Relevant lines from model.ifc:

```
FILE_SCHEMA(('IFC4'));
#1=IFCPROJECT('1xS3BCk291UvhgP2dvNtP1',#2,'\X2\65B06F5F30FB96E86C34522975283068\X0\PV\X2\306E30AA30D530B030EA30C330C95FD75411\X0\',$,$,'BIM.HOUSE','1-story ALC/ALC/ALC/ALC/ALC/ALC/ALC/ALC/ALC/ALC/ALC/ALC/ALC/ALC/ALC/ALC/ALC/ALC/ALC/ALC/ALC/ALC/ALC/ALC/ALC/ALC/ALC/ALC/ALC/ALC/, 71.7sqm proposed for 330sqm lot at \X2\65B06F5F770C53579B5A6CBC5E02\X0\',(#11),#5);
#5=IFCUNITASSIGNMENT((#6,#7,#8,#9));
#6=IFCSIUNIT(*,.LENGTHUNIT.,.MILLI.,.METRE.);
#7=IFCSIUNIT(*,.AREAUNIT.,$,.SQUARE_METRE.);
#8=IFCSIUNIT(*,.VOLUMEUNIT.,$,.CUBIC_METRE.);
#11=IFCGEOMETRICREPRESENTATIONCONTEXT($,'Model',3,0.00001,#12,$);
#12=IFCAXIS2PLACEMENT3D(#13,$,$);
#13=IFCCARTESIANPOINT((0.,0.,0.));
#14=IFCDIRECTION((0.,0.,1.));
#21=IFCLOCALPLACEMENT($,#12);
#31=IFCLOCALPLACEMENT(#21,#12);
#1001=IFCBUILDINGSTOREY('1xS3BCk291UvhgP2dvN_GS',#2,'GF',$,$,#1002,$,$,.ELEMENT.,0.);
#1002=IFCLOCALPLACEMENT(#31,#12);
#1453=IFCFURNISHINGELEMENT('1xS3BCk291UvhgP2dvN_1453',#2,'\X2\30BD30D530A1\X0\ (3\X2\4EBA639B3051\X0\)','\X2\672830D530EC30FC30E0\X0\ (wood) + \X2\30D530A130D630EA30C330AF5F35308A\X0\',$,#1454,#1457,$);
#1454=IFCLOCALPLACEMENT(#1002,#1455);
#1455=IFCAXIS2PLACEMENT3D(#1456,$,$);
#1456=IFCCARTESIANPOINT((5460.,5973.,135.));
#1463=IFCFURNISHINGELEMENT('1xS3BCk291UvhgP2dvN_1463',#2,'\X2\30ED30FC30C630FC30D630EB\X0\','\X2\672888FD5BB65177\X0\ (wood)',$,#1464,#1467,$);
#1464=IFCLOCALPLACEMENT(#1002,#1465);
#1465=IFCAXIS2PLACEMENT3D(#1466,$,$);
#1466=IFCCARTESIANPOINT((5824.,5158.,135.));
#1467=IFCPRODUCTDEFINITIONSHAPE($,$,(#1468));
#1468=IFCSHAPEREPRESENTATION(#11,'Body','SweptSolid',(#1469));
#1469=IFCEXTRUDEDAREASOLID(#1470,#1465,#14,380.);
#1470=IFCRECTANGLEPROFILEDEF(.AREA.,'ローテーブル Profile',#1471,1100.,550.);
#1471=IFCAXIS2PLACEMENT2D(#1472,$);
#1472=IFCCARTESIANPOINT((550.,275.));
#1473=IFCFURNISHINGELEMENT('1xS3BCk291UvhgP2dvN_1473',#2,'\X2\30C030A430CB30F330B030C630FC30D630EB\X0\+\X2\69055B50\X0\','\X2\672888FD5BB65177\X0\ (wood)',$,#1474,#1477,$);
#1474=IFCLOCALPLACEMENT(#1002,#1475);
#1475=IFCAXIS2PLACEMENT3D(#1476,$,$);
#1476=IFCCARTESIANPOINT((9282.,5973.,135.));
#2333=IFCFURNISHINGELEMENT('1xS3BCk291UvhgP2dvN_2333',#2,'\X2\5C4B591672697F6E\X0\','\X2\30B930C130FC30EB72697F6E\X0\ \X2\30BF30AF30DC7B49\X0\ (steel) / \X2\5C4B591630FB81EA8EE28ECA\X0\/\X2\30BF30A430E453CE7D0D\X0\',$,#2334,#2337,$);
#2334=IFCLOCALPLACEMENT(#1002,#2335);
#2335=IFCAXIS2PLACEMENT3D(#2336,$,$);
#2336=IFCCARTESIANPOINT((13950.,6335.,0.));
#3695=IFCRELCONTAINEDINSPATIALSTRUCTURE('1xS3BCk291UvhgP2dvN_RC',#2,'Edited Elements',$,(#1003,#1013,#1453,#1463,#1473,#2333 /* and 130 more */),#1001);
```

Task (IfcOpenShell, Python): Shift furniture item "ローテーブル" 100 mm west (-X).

```python
import ifcopenshell
import ifcopenshell.api.geometry
import ifcopenshell.util.placement
import ifcopenshell.util.unit

model = ifcopenshell.open("model.ifc")
unit_scale = ifcopenshell.util.unit.calculate_unit_scale(model)

item = model.by_id(1463)
matrix = ifcopenshell.util.placement.get_local_placement(item.ObjectPlacement)
matrix[0, 3] -= 0.1 / unit_scale
ifcopenshell.api.geometry.edit_object_placement(model, product=item, matrix=matrix, is_si=False)

print(ifcopenshell.util.placement.get_local_placement(item.ObjectPlacement).round(3) + 0.0)

model.write("model_edited.ifc")
```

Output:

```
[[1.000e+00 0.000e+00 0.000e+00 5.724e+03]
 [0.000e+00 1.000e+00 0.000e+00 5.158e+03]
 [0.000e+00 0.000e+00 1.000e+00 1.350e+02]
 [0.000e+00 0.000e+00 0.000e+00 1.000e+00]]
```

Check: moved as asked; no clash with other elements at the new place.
